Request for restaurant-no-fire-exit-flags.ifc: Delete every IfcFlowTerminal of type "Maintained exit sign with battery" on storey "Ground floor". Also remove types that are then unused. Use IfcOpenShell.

First a look at what the model holds.

```python
import ifcopenshell
import ifcopenshell.util.element

model = ifcopenshell.open("restaurant-no-fire-exit-flags.ifc")
print(model.schema)
storey = next(s for s in model.by_type("IfcBuildingStorey") if s.Name == "Ground floor")
terminals = [e for e in ifcopenshell.util.element.get_decomposition(storey) if e.is_a("IfcFlowTerminal")]
seen = {}
for e in terminals:
    element_type = ifcopenshell.util.element.get_type(e)
    name = element_type.Name if element_type not in (None, e) else None
    seen[name] = seen.get(name, 0) + 1
for name, count in sorted(seen.items(), key=str):
    print(count, "x", name)
```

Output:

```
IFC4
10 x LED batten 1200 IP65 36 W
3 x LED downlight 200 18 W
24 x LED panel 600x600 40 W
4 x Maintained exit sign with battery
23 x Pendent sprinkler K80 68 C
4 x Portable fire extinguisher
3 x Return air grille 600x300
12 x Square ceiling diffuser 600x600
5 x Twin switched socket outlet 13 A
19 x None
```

```python
import ifcopenshell
import ifcopenshell.api.root
import ifcopenshell.util.element

model = ifcopenshell.open("restaurant-no-fire-exit-flags.ifc")

storey = next(s for s in model.by_type("IfcBuildingStorey") if s.Name == "Ground floor")
terminals = [e for e in ifcopenshell.util.element.get_decomposition(storey) if e.is_a("IfcFlowTerminal")]
targets = [e for e in terminals if (t := ifcopenshell.util.element.get_type(e)) not in (None, e) and t.Name == "Maintained exit sign with battery"]
types = {ifcopenshell.util.element.get_type(e) for e in targets} - {None, *targets}

for e in targets:
    ifcopenshell.api.root.remove_product(model, product=e)
print(len(targets), "removed")

unused = [t for t in types if not ifcopenshell.util.element.get_types(t)]
for t in unused:
    ifcopenshell.api.root.remove_product(model, product=t)
print(len(unused), "unused types removed")

model.write("restaurant-no-fire-exit-flags_v2.ifc")
```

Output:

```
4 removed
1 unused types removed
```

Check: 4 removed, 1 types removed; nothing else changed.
